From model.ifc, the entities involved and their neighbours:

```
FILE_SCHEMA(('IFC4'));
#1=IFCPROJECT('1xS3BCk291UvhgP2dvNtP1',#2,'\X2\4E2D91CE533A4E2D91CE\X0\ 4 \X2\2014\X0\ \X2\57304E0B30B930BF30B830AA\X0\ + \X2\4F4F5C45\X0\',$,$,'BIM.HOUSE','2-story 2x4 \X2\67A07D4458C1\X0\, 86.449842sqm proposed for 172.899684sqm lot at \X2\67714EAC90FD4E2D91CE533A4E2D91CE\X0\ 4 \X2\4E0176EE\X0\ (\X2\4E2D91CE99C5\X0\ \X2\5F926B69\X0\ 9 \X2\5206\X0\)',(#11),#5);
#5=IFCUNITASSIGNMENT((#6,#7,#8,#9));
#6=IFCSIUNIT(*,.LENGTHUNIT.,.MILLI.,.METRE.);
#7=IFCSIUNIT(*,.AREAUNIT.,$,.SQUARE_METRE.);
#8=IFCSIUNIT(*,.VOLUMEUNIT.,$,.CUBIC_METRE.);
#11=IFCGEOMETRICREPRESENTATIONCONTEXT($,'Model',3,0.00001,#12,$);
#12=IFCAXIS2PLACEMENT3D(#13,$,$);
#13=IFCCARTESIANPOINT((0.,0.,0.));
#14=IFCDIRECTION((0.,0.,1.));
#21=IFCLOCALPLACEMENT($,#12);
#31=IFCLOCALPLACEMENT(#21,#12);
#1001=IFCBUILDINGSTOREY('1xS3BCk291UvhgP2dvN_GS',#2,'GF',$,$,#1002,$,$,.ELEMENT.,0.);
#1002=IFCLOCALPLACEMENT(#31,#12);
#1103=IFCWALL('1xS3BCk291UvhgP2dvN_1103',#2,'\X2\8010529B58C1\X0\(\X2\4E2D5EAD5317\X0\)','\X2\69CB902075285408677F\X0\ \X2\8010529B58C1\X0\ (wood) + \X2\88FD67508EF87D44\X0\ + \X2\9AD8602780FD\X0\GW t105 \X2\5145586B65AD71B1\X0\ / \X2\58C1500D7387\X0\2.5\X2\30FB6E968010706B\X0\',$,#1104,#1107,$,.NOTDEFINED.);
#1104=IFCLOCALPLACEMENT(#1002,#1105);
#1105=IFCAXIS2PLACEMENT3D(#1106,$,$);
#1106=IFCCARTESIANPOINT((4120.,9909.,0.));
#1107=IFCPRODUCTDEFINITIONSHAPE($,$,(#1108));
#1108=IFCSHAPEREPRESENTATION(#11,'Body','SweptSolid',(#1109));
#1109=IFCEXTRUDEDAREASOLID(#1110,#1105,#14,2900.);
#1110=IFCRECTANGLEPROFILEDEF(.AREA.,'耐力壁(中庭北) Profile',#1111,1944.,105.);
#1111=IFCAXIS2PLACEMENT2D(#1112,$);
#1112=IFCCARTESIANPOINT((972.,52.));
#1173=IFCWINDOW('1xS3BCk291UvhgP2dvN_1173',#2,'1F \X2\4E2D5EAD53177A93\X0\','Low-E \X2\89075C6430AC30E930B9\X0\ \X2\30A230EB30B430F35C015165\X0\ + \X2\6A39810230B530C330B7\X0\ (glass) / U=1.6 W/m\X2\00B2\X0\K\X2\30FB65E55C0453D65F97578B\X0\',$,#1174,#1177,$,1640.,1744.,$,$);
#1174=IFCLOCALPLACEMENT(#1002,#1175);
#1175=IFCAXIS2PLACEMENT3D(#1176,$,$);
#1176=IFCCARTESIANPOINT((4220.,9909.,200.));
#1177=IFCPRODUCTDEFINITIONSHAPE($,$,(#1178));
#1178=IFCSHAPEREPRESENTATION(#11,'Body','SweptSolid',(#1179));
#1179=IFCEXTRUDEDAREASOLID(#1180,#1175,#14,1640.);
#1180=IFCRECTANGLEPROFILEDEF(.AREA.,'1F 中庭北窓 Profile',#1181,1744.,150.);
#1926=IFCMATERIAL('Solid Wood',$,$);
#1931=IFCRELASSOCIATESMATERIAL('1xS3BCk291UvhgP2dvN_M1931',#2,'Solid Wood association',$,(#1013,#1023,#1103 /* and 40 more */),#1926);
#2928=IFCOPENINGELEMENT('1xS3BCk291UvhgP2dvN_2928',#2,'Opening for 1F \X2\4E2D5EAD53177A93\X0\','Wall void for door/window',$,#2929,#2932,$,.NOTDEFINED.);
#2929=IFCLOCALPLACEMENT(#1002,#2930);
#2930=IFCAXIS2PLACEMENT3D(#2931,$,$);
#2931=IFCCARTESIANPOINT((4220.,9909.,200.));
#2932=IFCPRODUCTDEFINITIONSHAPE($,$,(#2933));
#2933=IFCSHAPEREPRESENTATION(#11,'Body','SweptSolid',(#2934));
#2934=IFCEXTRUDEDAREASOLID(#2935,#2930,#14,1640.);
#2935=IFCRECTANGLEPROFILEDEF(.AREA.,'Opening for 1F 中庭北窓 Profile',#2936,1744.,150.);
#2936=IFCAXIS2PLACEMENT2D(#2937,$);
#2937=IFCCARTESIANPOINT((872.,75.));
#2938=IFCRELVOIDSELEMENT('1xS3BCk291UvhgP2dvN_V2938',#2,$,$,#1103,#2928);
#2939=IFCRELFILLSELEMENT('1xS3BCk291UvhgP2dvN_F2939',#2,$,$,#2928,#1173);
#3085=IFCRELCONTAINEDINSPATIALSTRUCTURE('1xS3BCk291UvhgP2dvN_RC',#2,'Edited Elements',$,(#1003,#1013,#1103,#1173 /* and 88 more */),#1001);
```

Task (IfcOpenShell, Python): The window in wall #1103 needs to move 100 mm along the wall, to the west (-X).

```python
import ifcopenshell
import ifcopenshell.api.geometry
import ifcopenshell.util.placement
import ifcopenshell.util.unit

model = ifcopenshell.open("model.ifc")
unit_scale = ifcopenshell.util.unit.calculate_unit_scale(model)

window = model.by_id(1173)
opening = window.FillsVoids[0].RelatingOpeningElement
wall = opening.VoidsElements[0].RelatingBuildingElement

wall_matrix = ifcopenshell.util.placement.get_local_placement(wall.ObjectPlacement)
shift = wall_matrix[:3, 0] * -0.1 / unit_scale
before = ifcopenshell.util.placement.get_local_placement(window.ObjectPlacement)[:3, 3].copy()

# The window is not placed relative to its opening, so move both.
for product in (opening, window):
    matrix = ifcopenshell.util.placement.get_local_placement(product.ObjectPlacement)
    matrix[:3, 3] += shift
    ifcopenshell.api.geometry.edit_object_placement(model, product=product, matrix=matrix, is_si=False)

after = ifcopenshell.util.placement.get_local_placement(window.ObjectPlacement)[:3, 3]
print("window moved by", (after - before).round(3) + 0.0)

model.write("model_edited.ifc")
```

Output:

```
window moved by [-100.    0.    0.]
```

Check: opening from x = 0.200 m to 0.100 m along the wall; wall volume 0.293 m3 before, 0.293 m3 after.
